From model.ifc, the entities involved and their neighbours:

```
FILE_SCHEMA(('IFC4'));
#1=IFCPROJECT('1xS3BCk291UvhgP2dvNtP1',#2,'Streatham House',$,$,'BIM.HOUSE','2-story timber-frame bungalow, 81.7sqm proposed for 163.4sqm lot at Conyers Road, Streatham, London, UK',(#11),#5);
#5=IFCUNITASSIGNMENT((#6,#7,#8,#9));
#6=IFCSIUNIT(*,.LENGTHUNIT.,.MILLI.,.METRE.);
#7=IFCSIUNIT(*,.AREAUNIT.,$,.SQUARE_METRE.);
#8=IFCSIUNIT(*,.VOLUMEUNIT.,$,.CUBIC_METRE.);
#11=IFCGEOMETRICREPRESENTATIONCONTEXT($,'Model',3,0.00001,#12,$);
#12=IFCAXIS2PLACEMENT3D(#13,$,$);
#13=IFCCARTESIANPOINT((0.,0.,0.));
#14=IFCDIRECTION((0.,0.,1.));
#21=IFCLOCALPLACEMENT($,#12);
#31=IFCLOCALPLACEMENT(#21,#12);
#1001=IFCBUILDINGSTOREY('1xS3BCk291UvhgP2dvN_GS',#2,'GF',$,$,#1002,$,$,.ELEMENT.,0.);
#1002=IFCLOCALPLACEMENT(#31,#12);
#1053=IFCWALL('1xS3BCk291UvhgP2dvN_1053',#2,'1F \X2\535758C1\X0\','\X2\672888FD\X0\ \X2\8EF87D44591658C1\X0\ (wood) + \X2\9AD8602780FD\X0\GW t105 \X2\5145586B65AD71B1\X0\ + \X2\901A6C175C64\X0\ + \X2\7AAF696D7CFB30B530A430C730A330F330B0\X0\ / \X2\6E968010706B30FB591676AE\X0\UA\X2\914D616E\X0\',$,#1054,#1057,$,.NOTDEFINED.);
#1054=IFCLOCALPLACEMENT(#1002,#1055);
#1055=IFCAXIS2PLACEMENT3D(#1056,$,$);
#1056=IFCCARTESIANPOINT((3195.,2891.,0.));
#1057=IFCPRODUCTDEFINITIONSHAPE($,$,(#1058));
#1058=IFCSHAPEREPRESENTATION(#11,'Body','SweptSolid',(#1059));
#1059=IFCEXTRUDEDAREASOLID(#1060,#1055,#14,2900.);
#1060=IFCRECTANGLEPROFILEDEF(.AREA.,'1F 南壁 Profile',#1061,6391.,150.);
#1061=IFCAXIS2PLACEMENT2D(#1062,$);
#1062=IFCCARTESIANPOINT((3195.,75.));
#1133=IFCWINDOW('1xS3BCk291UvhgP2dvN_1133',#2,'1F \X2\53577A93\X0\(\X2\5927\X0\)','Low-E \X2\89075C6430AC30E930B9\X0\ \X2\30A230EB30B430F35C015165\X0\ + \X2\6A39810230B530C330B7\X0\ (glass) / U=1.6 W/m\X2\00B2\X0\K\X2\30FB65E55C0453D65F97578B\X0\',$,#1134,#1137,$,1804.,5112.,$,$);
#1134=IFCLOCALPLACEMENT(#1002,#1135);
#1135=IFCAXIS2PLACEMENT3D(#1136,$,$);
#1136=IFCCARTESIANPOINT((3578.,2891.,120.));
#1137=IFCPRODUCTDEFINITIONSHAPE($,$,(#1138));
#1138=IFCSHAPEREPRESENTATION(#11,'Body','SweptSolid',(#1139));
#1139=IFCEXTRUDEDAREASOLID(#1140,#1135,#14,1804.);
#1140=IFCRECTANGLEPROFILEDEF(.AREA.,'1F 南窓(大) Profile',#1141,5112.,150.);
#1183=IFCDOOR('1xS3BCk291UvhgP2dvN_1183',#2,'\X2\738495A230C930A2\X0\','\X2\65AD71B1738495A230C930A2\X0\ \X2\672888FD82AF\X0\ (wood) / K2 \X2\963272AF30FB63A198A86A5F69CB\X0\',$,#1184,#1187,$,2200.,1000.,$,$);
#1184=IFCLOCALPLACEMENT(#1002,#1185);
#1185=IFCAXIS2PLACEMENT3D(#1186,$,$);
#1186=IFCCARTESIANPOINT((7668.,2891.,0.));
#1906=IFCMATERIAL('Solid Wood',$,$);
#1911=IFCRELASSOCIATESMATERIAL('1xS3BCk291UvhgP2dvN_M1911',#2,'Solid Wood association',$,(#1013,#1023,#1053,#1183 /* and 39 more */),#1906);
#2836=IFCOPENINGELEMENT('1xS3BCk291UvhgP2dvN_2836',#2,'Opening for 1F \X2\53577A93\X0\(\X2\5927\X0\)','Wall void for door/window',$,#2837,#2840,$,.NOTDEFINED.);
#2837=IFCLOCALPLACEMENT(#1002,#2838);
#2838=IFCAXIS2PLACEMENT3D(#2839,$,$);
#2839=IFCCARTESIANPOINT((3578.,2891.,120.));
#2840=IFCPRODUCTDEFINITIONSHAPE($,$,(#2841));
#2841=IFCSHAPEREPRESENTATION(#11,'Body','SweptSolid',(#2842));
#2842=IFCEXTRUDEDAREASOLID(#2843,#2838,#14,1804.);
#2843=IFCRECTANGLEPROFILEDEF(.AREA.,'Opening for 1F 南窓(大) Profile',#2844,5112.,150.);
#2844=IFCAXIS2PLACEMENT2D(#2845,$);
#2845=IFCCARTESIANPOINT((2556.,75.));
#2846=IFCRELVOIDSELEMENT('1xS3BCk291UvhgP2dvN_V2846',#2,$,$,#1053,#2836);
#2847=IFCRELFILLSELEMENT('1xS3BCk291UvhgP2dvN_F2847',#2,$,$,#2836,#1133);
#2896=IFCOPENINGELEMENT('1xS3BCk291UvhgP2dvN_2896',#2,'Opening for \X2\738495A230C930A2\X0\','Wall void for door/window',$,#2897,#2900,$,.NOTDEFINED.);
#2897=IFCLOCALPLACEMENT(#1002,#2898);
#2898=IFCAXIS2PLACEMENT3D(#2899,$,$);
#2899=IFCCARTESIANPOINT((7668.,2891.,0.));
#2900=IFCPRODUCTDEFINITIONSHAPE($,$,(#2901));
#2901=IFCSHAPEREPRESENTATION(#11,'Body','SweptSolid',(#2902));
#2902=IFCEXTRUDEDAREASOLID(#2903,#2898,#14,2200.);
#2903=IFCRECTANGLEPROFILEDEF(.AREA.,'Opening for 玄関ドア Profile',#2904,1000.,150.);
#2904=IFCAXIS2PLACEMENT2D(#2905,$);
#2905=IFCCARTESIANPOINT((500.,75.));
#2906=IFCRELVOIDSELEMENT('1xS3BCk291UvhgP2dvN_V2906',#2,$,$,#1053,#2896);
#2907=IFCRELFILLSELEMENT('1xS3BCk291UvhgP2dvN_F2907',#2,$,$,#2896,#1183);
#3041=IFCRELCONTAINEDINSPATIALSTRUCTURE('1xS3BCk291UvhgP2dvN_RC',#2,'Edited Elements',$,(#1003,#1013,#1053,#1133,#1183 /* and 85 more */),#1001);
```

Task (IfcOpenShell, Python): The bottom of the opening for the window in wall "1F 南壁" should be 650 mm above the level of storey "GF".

```python
import numpy as np
import ifcopenshell
import ifcopenshell.api.geometry
import ifcopenshell.geom
import ifcopenshell.util.element
import ifcopenshell.util.placement
import ifcopenshell.util.shape
import ifcopenshell.util.unit

model = ifcopenshell.open("model.ifc")
unit_scale = ifcopenshell.util.unit.calculate_unit_scale(model)

window = model.by_id(1133)
opening = window.FillsVoids[0].RelatingOpeningElement
storey = ifcopenshell.util.element.get_container(window, ifc_class="IfcBuildingStorey")
level = ifcopenshell.util.placement.get_local_placement(storey.ObjectPlacement)[2, 3]

# The opening's origin need not be at the sill, so measure its lowest point.
shape = ifcopenshell.geom.create_shape(ifcopenshell.geom.settings(), opening)
bottom = ifcopenshell.util.shape.get_shape_bottom_elevation(shape, shape.geometry) / unit_scale
dz = level + 0.65 / unit_scale - bottom

shift = np.array([0.0, 0.0, dz])
# The window is not placed relative to its opening, so move both.
for product in (opening, window):
    matrix = ifcopenshell.util.placement.get_local_placement(product.ObjectPlacement)
    matrix[:3, 3] += shift
    ifcopenshell.api.geometry.edit_object_placement(model, product=product, matrix=matrix, is_si=False)

print(f"moved by {dz * unit_scale:+.3f} m")

model.write("model_rev.ifc")
```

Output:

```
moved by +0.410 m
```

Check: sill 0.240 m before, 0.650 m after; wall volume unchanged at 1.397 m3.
